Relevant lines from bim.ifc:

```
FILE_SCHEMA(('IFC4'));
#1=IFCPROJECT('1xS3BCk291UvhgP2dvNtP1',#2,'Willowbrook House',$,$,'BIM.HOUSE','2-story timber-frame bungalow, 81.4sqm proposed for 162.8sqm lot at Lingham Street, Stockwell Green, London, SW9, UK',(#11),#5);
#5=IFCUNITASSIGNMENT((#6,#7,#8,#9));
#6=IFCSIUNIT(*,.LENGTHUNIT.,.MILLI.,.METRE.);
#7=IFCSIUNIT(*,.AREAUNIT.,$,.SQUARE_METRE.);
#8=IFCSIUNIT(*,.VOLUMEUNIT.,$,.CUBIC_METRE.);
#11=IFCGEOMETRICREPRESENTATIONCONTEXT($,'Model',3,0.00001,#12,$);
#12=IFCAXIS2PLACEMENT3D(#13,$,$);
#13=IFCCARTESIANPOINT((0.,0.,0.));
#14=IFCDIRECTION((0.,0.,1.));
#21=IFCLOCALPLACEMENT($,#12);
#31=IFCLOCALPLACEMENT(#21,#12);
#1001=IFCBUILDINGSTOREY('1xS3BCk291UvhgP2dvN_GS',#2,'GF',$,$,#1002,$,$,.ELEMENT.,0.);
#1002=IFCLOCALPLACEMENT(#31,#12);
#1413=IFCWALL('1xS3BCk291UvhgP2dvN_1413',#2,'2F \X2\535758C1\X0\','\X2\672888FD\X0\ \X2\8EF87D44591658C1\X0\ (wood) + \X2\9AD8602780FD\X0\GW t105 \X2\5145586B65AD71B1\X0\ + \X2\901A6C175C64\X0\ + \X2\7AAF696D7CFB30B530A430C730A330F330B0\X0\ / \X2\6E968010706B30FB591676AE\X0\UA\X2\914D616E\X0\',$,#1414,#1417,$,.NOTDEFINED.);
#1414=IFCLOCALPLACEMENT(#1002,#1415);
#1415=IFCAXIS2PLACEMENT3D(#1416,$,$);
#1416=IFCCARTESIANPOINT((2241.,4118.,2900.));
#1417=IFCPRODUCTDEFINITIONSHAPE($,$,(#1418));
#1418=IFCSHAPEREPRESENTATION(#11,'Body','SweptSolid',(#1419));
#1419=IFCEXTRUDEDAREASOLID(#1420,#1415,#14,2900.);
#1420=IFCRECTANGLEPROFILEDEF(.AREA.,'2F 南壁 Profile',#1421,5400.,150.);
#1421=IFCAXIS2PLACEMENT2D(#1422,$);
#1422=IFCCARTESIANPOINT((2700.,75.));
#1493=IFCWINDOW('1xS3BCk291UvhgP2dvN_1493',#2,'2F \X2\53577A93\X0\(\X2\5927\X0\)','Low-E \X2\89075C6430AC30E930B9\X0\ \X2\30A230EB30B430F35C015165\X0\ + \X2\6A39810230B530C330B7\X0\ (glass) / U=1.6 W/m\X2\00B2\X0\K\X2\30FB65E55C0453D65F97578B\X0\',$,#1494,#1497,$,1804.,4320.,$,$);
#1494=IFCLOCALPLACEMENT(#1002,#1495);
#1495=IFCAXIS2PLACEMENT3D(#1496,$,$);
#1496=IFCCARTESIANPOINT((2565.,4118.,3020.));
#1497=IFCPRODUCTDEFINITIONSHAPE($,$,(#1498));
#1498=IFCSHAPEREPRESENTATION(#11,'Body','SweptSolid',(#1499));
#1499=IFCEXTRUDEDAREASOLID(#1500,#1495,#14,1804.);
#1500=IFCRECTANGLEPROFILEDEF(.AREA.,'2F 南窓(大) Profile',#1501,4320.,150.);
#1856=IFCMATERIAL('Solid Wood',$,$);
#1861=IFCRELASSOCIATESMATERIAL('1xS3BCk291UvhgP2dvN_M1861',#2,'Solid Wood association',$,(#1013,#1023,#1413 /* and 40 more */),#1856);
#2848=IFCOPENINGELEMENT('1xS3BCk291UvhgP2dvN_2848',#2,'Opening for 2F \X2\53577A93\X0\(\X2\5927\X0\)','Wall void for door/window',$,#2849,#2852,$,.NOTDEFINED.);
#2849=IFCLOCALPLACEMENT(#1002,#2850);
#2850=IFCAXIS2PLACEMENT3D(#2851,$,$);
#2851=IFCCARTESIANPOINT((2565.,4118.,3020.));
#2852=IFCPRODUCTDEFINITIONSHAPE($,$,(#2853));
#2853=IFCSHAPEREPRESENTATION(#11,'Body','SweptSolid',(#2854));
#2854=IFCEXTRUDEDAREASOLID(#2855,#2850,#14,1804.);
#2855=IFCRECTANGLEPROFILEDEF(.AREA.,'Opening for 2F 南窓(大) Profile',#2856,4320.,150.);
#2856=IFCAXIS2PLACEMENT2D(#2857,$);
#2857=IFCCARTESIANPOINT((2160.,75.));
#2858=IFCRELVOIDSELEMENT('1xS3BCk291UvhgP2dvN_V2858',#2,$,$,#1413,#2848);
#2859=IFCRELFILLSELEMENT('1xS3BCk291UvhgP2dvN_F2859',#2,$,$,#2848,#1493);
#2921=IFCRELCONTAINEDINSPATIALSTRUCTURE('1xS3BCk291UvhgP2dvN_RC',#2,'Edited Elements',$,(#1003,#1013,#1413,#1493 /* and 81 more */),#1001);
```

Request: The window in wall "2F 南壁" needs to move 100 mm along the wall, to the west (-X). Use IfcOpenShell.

```python
import ifcopenshell
import ifcopenshell.api.geometry
import ifcopenshell.util.placement
import ifcopenshell.util.unit

model = ifcopenshell.open("bim.ifc")
unit_scale = ifcopenshell.util.unit.calculate_unit_scale(model)

window = model.by_id(1493)
opening = window.FillsVoids[0].RelatingOpeningElement
wall = opening.VoidsElements[0].RelatingBuildingElement

wall_matrix = ifcopenshell.util.placement.get_local_placement(wall.ObjectPlacement)
shift = wall_matrix[:3, 0] * -0.1 / unit_scale
before = ifcopenshell.util.placement.get_local_placement(window.ObjectPlacement)[:3, 3].copy()

# The window is not placed relative to its opening, so move both.
for product in (opening, window):
    matrix = ifcopenshell.util.placement.get_local_placement(product.ObjectPlacement)
    matrix[:3, 3] += shift
    ifcopenshell.api.geometry.edit_object_placement(model, product=product, matrix=matrix, is_si=False)

after = ifcopenshell.util.placement.get_local_placement(window.ObjectPlacement)[:3, 3]
print("window moved by", (after - before).round(3) + 0.0)

model.write("bim-out.ifc")
```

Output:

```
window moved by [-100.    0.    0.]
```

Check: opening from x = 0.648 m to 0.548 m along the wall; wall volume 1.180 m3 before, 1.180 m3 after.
